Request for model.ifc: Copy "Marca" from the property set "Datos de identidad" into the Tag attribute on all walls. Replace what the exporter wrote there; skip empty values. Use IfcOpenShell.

First a look at what the model holds.

```python
import ifcopenshell
import ifcopenshell.util.element

model = ifcopenshell.open("model.ifc")
print(model.schema)
walls = model.by_type("IfcWall")
print(len(walls), "walls")
for e in walls[:8]:
    source = ifcopenshell.util.element.get_pset(e, "Datos de identidad", "Marca")
    target = e.Tag
    print(e.id(), repr(source), repr(target), sep=" | ")
```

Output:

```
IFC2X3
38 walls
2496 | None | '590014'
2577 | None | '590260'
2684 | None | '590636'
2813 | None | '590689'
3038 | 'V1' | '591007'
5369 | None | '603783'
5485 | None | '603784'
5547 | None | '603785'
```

```python
import ifcopenshell
import ifcopenshell.util.element

model = ifcopenshell.open("model.ifc")

count = 0
for e in model.by_type("IfcWall"):
    value = ifcopenshell.util.element.get_pset(e, "Datos de identidad", "Marca")
    current = e.Tag
    if not value or not value.strip() or current == value:
        continue
    e.Tag = value
    count += 1

print(count, "walls updated")

model.write("model_updated.ifc")
```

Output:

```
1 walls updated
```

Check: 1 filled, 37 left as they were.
